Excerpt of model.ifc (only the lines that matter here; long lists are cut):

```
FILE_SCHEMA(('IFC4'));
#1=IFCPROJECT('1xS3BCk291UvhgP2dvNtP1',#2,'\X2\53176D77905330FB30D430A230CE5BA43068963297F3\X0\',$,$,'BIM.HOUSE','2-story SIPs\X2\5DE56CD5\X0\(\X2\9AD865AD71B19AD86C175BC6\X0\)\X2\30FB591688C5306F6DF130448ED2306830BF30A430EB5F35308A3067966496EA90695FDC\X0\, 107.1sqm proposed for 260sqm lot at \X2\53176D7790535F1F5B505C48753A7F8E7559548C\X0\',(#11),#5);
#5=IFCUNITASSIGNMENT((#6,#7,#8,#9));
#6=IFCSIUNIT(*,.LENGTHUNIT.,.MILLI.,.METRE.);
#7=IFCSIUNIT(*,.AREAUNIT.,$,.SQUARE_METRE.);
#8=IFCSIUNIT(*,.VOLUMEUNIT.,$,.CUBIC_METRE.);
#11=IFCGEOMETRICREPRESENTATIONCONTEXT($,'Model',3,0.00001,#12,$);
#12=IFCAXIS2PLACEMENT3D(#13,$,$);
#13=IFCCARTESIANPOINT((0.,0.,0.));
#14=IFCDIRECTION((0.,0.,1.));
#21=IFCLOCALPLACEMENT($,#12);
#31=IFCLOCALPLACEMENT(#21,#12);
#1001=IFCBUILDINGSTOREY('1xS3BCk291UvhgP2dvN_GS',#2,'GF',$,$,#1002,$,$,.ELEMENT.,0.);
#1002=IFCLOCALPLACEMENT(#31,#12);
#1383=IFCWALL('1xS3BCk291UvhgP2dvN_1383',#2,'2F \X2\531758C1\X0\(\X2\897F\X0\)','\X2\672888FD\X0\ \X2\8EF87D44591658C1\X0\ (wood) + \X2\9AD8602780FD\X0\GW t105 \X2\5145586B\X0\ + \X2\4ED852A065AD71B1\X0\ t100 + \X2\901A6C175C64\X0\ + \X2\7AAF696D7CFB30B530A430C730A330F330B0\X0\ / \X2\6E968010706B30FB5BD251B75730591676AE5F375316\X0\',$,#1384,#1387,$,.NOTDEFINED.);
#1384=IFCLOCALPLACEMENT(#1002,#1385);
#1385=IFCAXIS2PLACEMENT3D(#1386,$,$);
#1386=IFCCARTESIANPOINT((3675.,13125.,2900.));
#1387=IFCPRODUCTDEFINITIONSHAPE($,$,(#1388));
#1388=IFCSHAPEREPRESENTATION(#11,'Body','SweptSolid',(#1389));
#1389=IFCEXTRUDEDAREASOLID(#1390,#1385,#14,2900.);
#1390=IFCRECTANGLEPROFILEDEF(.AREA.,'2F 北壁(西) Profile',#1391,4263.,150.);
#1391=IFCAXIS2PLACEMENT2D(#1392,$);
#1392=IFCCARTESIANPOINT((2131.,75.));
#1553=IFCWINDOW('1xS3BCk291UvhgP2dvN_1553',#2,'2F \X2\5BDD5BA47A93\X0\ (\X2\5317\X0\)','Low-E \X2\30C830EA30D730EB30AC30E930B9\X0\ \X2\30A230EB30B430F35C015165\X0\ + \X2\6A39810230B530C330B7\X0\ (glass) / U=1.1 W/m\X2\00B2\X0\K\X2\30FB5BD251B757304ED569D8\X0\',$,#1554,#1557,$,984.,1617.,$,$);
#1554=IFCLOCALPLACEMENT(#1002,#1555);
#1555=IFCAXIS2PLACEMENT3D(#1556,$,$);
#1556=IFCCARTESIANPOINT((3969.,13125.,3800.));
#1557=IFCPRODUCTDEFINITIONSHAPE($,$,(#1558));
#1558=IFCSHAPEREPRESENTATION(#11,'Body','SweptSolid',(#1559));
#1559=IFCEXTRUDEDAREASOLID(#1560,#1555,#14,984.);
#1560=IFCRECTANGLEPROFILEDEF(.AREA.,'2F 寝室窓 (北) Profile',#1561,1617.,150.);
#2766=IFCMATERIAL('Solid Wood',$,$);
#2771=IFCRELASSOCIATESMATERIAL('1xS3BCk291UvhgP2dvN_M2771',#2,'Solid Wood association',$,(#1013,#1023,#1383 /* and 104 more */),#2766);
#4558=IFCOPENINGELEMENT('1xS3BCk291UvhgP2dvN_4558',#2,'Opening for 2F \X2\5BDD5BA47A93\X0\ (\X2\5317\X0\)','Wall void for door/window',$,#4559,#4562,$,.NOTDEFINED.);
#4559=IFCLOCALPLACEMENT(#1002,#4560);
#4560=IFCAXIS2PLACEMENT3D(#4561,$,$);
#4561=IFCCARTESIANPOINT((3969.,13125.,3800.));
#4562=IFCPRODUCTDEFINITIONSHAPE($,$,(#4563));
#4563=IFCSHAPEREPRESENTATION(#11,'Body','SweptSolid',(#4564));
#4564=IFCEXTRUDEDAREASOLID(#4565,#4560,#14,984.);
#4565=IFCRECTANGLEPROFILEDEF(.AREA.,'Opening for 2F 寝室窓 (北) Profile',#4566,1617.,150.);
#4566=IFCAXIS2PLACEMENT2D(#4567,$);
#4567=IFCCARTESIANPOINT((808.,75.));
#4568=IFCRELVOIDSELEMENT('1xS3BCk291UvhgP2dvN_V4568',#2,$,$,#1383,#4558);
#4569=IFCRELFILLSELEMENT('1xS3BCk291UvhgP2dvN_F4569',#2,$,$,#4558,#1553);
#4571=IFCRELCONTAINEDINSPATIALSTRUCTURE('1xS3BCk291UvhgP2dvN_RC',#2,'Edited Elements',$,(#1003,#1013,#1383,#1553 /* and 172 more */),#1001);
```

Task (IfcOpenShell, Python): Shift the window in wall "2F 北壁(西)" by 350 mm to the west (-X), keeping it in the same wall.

```python
import ifcopenshell
import ifcopenshell.api.geometry
import ifcopenshell.util.placement
import ifcopenshell.util.unit

model = ifcopenshell.open("model.ifc")
unit_scale = ifcopenshell.util.unit.calculate_unit_scale(model)

window = model.by_id(1553)
opening = window.FillsVoids[0].RelatingOpeningElement
wall = opening.VoidsElements[0].RelatingBuildingElement

wall_matrix = ifcopenshell.util.placement.get_local_placement(wall.ObjectPlacement)
shift = wall_matrix[:3, 0] * -0.35 / unit_scale
before = ifcopenshell.util.placement.get_local_placement(window.ObjectPlacement)[:3, 3].copy()

# The window is not placed relative to its opening, so move both.
for product in (opening, window):
    matrix = ifcopenshell.util.placement.get_local_placement(product.ObjectPlacement)
    matrix[:3, 3] += shift
    ifcopenshell.api.geometry.edit_object_placement(model, product=product, matrix=matrix, is_si=False)

after = ifcopenshell.util.placement.get_local_placement(window.ObjectPlacement)[:3, 3]
print("window moved by", (after - before).round(3) + 0.0)

model.write("model_updated.ifc")
```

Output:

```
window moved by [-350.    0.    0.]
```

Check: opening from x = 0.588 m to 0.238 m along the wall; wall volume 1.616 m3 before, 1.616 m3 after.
